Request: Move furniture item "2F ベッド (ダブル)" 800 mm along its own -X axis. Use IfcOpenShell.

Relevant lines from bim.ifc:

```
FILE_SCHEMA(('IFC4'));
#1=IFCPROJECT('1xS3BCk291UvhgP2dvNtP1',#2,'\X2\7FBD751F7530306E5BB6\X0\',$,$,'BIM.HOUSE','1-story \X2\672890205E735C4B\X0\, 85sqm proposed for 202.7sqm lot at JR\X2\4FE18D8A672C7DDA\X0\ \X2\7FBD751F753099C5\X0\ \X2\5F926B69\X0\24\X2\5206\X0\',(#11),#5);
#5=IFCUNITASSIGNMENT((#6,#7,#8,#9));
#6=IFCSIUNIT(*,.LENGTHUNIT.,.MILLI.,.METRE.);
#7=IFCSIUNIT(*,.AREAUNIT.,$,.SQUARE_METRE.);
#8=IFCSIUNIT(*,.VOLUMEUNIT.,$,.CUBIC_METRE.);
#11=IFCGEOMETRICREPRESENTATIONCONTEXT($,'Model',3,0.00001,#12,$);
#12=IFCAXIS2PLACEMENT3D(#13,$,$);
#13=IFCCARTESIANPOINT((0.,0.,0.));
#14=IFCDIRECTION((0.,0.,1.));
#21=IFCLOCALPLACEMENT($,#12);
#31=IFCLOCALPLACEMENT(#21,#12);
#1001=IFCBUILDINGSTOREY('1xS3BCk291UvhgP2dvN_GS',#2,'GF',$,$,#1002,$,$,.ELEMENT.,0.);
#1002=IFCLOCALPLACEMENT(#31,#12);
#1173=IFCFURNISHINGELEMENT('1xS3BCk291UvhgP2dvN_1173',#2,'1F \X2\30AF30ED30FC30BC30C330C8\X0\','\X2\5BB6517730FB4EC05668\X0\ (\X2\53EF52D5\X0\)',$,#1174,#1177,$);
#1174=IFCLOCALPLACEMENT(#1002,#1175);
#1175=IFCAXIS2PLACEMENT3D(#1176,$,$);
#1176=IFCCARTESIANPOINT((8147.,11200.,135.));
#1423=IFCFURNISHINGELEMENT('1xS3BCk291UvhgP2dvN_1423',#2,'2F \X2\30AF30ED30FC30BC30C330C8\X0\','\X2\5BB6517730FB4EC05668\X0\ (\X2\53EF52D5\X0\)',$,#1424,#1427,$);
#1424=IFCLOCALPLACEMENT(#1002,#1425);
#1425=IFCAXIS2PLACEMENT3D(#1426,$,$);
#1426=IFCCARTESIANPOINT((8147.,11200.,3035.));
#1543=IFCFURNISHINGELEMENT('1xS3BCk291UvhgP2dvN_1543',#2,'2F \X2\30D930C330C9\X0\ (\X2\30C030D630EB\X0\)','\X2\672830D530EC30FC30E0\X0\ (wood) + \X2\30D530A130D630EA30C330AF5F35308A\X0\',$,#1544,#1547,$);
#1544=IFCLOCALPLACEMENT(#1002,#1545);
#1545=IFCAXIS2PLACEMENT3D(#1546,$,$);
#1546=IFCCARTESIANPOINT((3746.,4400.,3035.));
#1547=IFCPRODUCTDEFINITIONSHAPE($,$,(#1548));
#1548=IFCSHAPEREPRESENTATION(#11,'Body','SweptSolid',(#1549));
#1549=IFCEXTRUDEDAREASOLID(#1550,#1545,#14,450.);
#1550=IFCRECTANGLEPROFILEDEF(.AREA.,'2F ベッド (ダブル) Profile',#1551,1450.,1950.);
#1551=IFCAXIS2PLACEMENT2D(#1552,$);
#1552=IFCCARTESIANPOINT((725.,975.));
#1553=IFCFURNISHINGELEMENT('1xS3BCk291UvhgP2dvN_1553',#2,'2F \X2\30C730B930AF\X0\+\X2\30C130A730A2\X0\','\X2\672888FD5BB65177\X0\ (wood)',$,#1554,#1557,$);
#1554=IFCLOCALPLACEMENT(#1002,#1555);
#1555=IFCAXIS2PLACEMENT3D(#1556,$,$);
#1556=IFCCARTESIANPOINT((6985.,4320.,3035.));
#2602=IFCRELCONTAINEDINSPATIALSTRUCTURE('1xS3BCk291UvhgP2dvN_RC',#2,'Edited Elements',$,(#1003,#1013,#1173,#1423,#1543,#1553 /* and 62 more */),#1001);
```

```python
import ifcopenshell
import ifcopenshell.api.geometry
import ifcopenshell.util.placement
import ifcopenshell.util.unit

model = ifcopenshell.open("bim.ifc")
unit_scale = ifcopenshell.util.unit.calculate_unit_scale(model)

item = model.by_guid("1xS3BCk291UvhgP2dvN_1543")
matrix = ifcopenshell.util.placement.get_local_placement(item.ObjectPlacement)
matrix[:3, 3] -= matrix[:3, 0] * 0.8 / unit_scale
ifcopenshell.api.geometry.edit_object_placement(model, product=item, matrix=matrix, is_si=False)

print(ifcopenshell.util.placement.get_local_placement(item.ObjectPlacement).round(3) + 0.0)

model.write("bim_v2.ifc")
```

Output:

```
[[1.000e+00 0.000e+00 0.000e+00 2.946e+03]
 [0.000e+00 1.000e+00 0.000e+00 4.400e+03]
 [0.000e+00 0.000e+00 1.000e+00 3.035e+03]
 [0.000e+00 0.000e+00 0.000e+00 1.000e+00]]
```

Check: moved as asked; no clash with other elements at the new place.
